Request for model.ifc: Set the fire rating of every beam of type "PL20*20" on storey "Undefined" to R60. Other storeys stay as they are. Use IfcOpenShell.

First a look at what the model holds.

```python
import ifcopenshell
import ifcopenshell.util.element

model = ifcopenshell.open("model.ifc")
print(model.schema)
storey = next(s for s in model.by_type("IfcBuildingStorey") if s.Name == "Undefined")
beams = [e for e in ifcopenshell.util.element.get_decomposition(storey) if e.is_a("IfcBeam")]
seen = {}
for e in beams:
    element_type = ifcopenshell.util.element.get_type(e)
    key = (element_type.Name if element_type != e and element_type else None, ifcopenshell.util.element.get_pset(e, "Pset_BeamCommon", "FireRating"))
    seen[key] = seen.get(key, 0) + 1
for (name, value), count in sorted(seen.items(), key=str):
    print(count, "x", name, "|", value)
```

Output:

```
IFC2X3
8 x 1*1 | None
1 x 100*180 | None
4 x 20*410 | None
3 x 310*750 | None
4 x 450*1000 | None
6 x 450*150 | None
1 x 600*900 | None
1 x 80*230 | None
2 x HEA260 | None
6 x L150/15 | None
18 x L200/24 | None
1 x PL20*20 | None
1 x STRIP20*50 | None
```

```python
import ifcopenshell
import ifcopenshell.api.pset
import ifcopenshell.util.element

model = ifcopenshell.open("model.ifc")

storey = next(s for s in model.by_type("IfcBuildingStorey") if s.Name == "Undefined")
beams = [e for e in ifcopenshell.util.element.get_decomposition(storey) if e.is_a("IfcBeam")]

count = 0
for e in beams:
    element_type = ifcopenshell.util.element.get_type(e)
    if element_type in (None, e) or element_type.Name != "PL20*20":
        continue
    found = ifcopenshell.util.element.get_pset(e, "Pset_BeamCommon", should_inherit=False)
    if found:
        pset = model.by_id(found["id"])
        if len(ifcopenshell.util.element.get_elements_by_pset(pset)) > 1:
            pset = ifcopenshell.api.pset.unshare_pset(model, products=[e], pset=pset)[0]
    else:
        pset = ifcopenshell.api.pset.add_pset(model, product=e, name="Pset_BeamCommon")
    ifcopenshell.api.pset.edit_pset(model, pset=pset, properties={"FireRating": "R60"})
    count += 1

print(count, "beams updated")

model.write("model_updated.ifc")
```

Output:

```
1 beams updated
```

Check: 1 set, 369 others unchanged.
